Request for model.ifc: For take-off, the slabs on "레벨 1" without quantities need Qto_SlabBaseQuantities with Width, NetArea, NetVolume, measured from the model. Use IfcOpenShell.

First a look at what the model holds.

```python
import ifcopenshell
import ifcopenshell.util.element
import ifcopenshell.util.unit

model = ifcopenshell.open("model.ifc")
print(model.schema)
for unit_type in ("LENGTHUNIT", "AREAUNIT", "VOLUMEUNIT"):
    print(unit_type, ifcopenshell.util.unit.calculate_unit_scale(model, unit_type))
storey = next(s for s in model.by_type("IfcBuildingStorey") if s.Name == "레벨 1")
slabs = [e for e in ifcopenshell.util.element.get_decomposition(storey) if e.is_a("IfcSlab")]
for e in sorted(slabs, key=lambda e: e.id()):
    print(e.id(), e.is_a(), e.Name, list(ifcopenshell.util.element.get_psets(e, qtos_only=True)), sep=" | ")
```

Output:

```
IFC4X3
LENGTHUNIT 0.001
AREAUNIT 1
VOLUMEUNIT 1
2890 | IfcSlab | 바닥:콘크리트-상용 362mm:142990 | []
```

```python
import ifcopenshell
import ifcopenshell.api.pset
import ifcopenshell.geom
import ifcopenshell.util.element
import ifcopenshell.util.shape
import ifcopenshell.util.unit

model = ifcopenshell.open("model.ifc")
unit_scale = ifcopenshell.util.unit.calculate_unit_scale(model)
area_scale = ifcopenshell.util.unit.calculate_unit_scale(model, "AREAUNIT")
volume_scale = ifcopenshell.util.unit.calculate_unit_scale(model, "VOLUMEUNIT")
settings = ifcopenshell.geom.settings()

storey = next(s for s in model.by_type("IfcBuildingStorey") if s.Name == "레벨 1")
slabs = [e for e in ifcopenshell.util.element.get_decomposition(storey) if e.is_a("IfcSlab")]

for e in sorted(slabs, key=lambda e: e.id()):
    if ifcopenshell.util.element.get_psets(e, qtos_only=True, should_inherit=False):
        continue
    # Geometry comes back in metres, in the element's own axes.
    shape = ifcopenshell.geom.create_shape(settings, e)
    values = {
        "Width": ifcopenshell.util.shape.get_z(shape.geometry) / unit_scale,
        "NetArea": ifcopenshell.util.shape.get_footprint_area(shape.geometry) / area_scale,
        "NetVolume": ifcopenshell.util.shape.get_volume(shape.geometry) / volume_scale,
    }
    qto = ifcopenshell.api.pset.add_qto(model, product=e, name="Qto_SlabBaseQuantities")
    ifcopenshell.api.pset.edit_qto(model, qto=qto, properties=values)
    print(e.id(), {k: round(v, 3) for k, v in values.items()})

model.write("model_updated.ifc")
```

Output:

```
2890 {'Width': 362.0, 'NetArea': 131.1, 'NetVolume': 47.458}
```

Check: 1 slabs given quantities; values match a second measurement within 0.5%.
